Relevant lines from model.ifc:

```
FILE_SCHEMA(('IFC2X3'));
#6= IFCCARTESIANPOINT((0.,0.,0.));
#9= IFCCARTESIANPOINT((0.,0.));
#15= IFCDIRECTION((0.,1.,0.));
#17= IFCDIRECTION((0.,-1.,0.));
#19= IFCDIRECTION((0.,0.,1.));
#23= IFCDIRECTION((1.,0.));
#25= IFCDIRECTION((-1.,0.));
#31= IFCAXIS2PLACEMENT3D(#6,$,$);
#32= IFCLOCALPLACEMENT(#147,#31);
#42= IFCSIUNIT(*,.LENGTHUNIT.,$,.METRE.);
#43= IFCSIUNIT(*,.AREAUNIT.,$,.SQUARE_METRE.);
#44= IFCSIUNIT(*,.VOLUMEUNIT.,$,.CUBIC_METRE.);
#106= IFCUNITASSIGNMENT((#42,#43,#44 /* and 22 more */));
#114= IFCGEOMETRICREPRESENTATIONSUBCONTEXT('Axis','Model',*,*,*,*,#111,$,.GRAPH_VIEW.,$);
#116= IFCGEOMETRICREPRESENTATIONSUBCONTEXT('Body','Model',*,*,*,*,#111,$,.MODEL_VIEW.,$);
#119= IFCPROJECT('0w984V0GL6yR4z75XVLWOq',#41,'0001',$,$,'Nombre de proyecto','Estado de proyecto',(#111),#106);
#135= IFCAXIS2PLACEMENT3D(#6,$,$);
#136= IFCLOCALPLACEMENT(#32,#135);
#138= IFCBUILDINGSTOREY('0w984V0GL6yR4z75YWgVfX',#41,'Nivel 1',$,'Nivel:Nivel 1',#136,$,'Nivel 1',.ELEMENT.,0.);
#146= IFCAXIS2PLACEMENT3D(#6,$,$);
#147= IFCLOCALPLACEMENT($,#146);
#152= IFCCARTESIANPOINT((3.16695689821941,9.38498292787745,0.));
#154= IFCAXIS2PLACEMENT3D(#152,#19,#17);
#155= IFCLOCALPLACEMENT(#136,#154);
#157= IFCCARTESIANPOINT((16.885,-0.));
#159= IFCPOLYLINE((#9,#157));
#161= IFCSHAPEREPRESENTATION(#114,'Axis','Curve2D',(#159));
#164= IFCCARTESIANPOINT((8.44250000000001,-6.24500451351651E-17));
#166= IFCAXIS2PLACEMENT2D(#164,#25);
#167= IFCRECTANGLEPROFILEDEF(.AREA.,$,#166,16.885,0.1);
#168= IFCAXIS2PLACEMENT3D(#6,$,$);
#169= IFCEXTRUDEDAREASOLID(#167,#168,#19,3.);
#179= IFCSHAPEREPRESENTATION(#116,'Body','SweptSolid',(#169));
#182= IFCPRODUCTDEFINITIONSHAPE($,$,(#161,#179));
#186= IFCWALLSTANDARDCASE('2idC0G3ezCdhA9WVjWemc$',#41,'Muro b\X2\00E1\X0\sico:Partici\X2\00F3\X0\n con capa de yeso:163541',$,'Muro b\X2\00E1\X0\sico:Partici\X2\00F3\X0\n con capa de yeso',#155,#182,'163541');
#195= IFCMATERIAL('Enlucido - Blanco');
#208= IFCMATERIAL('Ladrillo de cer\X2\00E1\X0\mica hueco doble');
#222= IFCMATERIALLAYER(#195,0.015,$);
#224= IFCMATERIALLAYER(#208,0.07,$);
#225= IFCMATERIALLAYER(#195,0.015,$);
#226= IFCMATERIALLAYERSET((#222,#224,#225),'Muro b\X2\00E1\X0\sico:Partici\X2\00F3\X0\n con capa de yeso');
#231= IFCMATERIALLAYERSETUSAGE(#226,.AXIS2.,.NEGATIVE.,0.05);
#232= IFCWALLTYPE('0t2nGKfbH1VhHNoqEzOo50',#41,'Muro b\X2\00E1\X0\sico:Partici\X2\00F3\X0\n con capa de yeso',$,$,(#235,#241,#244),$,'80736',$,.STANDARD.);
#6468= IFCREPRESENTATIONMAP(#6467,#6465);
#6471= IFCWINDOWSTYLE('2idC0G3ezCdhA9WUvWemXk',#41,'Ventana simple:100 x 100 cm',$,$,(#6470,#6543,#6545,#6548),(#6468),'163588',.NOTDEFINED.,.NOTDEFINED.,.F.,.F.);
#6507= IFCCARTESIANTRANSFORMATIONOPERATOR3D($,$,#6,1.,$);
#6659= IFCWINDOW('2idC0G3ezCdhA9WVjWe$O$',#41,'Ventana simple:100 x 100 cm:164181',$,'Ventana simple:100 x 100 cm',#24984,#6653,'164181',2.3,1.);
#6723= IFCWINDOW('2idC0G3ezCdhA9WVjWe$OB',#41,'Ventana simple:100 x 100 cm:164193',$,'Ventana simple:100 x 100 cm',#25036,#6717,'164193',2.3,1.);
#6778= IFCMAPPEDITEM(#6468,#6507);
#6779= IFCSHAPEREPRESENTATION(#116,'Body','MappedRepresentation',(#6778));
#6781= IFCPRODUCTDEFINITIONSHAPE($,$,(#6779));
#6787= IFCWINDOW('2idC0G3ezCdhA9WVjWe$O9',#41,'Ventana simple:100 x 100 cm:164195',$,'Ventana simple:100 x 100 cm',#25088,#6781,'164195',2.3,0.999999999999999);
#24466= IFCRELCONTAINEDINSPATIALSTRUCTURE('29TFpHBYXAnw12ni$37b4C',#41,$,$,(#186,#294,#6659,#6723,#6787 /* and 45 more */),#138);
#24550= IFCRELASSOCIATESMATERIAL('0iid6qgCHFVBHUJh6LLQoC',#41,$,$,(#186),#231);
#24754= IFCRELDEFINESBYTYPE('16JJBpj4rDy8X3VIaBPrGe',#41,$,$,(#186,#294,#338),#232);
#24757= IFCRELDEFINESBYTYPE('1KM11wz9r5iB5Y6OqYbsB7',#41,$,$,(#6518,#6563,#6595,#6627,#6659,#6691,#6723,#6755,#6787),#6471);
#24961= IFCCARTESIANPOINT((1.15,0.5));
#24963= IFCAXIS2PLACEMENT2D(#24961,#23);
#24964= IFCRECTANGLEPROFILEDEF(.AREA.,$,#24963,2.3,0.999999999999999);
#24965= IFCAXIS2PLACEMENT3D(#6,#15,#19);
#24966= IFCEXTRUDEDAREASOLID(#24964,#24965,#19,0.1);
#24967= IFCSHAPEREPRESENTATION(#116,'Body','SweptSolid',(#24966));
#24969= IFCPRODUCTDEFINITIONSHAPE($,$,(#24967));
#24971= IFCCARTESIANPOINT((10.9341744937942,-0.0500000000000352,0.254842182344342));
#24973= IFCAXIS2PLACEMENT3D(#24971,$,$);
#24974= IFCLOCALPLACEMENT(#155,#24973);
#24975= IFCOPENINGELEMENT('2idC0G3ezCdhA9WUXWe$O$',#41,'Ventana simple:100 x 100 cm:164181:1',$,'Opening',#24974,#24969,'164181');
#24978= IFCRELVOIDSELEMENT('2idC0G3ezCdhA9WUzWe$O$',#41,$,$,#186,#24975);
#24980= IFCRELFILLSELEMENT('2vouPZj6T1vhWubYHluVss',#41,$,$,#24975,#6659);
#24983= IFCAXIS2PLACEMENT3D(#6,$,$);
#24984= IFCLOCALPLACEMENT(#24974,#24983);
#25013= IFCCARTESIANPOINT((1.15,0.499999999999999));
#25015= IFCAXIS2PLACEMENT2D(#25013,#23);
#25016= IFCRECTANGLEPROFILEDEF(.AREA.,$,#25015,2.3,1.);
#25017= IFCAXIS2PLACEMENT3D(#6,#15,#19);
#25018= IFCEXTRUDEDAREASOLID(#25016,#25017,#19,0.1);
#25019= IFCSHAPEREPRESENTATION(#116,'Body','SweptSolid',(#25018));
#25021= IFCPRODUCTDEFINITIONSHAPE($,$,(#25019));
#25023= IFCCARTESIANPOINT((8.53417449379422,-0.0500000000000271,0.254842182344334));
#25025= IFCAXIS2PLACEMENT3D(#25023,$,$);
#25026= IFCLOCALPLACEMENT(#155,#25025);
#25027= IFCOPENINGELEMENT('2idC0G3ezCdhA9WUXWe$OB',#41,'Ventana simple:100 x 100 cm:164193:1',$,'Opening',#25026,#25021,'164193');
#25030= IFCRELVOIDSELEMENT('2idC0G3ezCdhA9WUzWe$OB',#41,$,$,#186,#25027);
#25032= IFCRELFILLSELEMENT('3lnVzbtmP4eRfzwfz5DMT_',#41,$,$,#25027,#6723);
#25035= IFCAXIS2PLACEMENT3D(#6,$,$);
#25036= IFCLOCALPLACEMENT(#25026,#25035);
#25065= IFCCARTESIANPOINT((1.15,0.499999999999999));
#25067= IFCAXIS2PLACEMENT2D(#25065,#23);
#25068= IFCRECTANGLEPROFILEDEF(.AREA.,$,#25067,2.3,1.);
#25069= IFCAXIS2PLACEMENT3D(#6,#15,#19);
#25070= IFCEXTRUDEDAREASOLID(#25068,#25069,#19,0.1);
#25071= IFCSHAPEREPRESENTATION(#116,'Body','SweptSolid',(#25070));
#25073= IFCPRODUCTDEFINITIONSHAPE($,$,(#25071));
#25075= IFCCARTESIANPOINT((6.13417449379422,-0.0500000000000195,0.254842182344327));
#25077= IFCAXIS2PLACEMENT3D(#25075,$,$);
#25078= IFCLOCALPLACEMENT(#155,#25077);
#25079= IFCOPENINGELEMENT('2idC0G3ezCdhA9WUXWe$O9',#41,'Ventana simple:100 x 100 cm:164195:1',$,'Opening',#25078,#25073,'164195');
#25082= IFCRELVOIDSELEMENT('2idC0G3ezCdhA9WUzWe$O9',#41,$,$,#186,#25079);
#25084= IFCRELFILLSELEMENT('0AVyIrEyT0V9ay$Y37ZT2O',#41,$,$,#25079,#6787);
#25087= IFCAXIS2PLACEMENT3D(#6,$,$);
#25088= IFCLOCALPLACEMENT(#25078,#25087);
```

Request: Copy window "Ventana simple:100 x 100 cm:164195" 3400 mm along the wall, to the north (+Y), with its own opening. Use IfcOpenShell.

```python
import ifcopenshell
import ifcopenshell.api.feature
import ifcopenshell.api.geometry
import ifcopenshell.api.root
import ifcopenshell.geom
import ifcopenshell.util.element
import ifcopenshell.util.placement
import ifcopenshell.util.shape
import ifcopenshell.util.unit

model = ifcopenshell.open("model.ifc")
unit_scale = ifcopenshell.util.unit.calculate_unit_scale(model)
settings = ifcopenshell.geom.settings()


def volume(element):
    """Net volume in cubic metres, openings subtracted."""
    shape = ifcopenshell.geom.create_shape(settings, element)
    return ifcopenshell.util.shape.get_volume(shape.geometry)


def reuse_history(source, copy):
    """copy_class also copies each property set's owner history, people and application; keep the originals."""
    for rel in copy.IsDefinedBy:
        if rel.is_a("IfcRelDefinesByProperties") and (history := rel.RelatingPropertyDefinition.OwnerHistory):
            rel.RelatingPropertyDefinition.OwnerHistory = source.OwnerHistory
            ifcopenshell.util.element.remove_deep2(model, history)


window = model.by_guid("2idC0G3ezCdhA9WVjWe$O9")
opening = window.FillsVoids[0].RelatingOpeningElement
wall = opening.VoidsElements[0].RelatingBuildingElement
before = volume(wall)
shift = ifcopenshell.util.placement.get_local_placement(wall.ObjectPlacement)[:3, 0] * -3.4 / unit_scale

# copy_class copies the void relationship, type, container and properties, but no geometry.
new_opening = ifcopenshell.api.root.copy_class(model, product=opening)
new_opening.Representation = ifcopenshell.util.element.copy_deep(
    model, opening.Representation, exclude=["IfcGeometricRepresentationContext", "IfcRepresentationMap"]
)
new_opening.Name = "Ventana simple:100 x 100 cm"
new_opening.Tag = None
new_window = ifcopenshell.api.root.copy_class(model, product=window)
new_window.Representation = ifcopenshell.util.element.copy_deep(
    model, window.Representation, exclude=["IfcGeometricRepresentationContext", "IfcRepresentationMap"]
)
new_window.Name = "Ventana simple:100 x 100 cm"
new_window.Tag = None
reuse_history(window, new_window)
fills = ifcopenshell.api.feature.add_filling(model, opening=new_opening, element=new_window)
fills.OwnerHistory = new_window.OwnerHistory  # required in IFC2X3

for old, new in ((opening, new_opening), (window, new_window)):
    matrix = ifcopenshell.util.placement.get_local_placement(old.ObjectPlacement)
    matrix[:3, 3] += shift
    ifcopenshell.api.geometry.edit_object_placement(model, product=new, matrix=matrix, is_si=False)

after = volume(wall)

print(f"wall volume {before:.3f} -> {after:.3f} m3")

model.write("model_v2.ifc")
```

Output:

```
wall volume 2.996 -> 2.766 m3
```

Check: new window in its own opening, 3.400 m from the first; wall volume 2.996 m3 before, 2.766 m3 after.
